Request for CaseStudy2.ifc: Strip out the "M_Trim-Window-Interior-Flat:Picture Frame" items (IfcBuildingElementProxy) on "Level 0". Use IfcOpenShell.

First a look at what the model holds.

```python
import ifcopenshell
import ifcopenshell.util.element

model = ifcopenshell.open("CaseStudy2.ifc")
print(model.schema)
storey = next(s for s in model.by_type("IfcBuildingStorey") if s.Name == "Level 0")
proxies = [e for e in ifcopenshell.util.element.get_decomposition(storey) if e.is_a("IfcBuildingElementProxy")]
seen = {}
for e in proxies:
    element_type = ifcopenshell.util.element.get_type(e)
    name = element_type.Name if element_type not in (None, e) else None
    seen[name] = seen.get(name, 0) + 1
for name, count in sorted(seen.items(), key=str):
    print(count, "x", name)
```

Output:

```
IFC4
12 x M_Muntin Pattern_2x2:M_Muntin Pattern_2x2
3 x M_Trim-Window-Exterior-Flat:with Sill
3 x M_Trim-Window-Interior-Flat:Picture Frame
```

```python
import ifcopenshell
import ifcopenshell.api.root
import ifcopenshell.util.element

model = ifcopenshell.open("CaseStudy2.ifc")

storey = next(s for s in model.by_type("IfcBuildingStorey") if s.Name == "Level 0")
proxies = [e for e in ifcopenshell.util.element.get_decomposition(storey) if e.is_a("IfcBuildingElementProxy")]
targets = [e for e in proxies if (t := ifcopenshell.util.element.get_type(e)) not in (None, e) and t.Name == "M_Trim-Window-Interior-Flat:Picture Frame"]

for e in targets:
    ifcopenshell.api.root.remove_product(model, product=e)
print(len(targets), "removed")

model.write("CaseStudy2_v2.ifc")
```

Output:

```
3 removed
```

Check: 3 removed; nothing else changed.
